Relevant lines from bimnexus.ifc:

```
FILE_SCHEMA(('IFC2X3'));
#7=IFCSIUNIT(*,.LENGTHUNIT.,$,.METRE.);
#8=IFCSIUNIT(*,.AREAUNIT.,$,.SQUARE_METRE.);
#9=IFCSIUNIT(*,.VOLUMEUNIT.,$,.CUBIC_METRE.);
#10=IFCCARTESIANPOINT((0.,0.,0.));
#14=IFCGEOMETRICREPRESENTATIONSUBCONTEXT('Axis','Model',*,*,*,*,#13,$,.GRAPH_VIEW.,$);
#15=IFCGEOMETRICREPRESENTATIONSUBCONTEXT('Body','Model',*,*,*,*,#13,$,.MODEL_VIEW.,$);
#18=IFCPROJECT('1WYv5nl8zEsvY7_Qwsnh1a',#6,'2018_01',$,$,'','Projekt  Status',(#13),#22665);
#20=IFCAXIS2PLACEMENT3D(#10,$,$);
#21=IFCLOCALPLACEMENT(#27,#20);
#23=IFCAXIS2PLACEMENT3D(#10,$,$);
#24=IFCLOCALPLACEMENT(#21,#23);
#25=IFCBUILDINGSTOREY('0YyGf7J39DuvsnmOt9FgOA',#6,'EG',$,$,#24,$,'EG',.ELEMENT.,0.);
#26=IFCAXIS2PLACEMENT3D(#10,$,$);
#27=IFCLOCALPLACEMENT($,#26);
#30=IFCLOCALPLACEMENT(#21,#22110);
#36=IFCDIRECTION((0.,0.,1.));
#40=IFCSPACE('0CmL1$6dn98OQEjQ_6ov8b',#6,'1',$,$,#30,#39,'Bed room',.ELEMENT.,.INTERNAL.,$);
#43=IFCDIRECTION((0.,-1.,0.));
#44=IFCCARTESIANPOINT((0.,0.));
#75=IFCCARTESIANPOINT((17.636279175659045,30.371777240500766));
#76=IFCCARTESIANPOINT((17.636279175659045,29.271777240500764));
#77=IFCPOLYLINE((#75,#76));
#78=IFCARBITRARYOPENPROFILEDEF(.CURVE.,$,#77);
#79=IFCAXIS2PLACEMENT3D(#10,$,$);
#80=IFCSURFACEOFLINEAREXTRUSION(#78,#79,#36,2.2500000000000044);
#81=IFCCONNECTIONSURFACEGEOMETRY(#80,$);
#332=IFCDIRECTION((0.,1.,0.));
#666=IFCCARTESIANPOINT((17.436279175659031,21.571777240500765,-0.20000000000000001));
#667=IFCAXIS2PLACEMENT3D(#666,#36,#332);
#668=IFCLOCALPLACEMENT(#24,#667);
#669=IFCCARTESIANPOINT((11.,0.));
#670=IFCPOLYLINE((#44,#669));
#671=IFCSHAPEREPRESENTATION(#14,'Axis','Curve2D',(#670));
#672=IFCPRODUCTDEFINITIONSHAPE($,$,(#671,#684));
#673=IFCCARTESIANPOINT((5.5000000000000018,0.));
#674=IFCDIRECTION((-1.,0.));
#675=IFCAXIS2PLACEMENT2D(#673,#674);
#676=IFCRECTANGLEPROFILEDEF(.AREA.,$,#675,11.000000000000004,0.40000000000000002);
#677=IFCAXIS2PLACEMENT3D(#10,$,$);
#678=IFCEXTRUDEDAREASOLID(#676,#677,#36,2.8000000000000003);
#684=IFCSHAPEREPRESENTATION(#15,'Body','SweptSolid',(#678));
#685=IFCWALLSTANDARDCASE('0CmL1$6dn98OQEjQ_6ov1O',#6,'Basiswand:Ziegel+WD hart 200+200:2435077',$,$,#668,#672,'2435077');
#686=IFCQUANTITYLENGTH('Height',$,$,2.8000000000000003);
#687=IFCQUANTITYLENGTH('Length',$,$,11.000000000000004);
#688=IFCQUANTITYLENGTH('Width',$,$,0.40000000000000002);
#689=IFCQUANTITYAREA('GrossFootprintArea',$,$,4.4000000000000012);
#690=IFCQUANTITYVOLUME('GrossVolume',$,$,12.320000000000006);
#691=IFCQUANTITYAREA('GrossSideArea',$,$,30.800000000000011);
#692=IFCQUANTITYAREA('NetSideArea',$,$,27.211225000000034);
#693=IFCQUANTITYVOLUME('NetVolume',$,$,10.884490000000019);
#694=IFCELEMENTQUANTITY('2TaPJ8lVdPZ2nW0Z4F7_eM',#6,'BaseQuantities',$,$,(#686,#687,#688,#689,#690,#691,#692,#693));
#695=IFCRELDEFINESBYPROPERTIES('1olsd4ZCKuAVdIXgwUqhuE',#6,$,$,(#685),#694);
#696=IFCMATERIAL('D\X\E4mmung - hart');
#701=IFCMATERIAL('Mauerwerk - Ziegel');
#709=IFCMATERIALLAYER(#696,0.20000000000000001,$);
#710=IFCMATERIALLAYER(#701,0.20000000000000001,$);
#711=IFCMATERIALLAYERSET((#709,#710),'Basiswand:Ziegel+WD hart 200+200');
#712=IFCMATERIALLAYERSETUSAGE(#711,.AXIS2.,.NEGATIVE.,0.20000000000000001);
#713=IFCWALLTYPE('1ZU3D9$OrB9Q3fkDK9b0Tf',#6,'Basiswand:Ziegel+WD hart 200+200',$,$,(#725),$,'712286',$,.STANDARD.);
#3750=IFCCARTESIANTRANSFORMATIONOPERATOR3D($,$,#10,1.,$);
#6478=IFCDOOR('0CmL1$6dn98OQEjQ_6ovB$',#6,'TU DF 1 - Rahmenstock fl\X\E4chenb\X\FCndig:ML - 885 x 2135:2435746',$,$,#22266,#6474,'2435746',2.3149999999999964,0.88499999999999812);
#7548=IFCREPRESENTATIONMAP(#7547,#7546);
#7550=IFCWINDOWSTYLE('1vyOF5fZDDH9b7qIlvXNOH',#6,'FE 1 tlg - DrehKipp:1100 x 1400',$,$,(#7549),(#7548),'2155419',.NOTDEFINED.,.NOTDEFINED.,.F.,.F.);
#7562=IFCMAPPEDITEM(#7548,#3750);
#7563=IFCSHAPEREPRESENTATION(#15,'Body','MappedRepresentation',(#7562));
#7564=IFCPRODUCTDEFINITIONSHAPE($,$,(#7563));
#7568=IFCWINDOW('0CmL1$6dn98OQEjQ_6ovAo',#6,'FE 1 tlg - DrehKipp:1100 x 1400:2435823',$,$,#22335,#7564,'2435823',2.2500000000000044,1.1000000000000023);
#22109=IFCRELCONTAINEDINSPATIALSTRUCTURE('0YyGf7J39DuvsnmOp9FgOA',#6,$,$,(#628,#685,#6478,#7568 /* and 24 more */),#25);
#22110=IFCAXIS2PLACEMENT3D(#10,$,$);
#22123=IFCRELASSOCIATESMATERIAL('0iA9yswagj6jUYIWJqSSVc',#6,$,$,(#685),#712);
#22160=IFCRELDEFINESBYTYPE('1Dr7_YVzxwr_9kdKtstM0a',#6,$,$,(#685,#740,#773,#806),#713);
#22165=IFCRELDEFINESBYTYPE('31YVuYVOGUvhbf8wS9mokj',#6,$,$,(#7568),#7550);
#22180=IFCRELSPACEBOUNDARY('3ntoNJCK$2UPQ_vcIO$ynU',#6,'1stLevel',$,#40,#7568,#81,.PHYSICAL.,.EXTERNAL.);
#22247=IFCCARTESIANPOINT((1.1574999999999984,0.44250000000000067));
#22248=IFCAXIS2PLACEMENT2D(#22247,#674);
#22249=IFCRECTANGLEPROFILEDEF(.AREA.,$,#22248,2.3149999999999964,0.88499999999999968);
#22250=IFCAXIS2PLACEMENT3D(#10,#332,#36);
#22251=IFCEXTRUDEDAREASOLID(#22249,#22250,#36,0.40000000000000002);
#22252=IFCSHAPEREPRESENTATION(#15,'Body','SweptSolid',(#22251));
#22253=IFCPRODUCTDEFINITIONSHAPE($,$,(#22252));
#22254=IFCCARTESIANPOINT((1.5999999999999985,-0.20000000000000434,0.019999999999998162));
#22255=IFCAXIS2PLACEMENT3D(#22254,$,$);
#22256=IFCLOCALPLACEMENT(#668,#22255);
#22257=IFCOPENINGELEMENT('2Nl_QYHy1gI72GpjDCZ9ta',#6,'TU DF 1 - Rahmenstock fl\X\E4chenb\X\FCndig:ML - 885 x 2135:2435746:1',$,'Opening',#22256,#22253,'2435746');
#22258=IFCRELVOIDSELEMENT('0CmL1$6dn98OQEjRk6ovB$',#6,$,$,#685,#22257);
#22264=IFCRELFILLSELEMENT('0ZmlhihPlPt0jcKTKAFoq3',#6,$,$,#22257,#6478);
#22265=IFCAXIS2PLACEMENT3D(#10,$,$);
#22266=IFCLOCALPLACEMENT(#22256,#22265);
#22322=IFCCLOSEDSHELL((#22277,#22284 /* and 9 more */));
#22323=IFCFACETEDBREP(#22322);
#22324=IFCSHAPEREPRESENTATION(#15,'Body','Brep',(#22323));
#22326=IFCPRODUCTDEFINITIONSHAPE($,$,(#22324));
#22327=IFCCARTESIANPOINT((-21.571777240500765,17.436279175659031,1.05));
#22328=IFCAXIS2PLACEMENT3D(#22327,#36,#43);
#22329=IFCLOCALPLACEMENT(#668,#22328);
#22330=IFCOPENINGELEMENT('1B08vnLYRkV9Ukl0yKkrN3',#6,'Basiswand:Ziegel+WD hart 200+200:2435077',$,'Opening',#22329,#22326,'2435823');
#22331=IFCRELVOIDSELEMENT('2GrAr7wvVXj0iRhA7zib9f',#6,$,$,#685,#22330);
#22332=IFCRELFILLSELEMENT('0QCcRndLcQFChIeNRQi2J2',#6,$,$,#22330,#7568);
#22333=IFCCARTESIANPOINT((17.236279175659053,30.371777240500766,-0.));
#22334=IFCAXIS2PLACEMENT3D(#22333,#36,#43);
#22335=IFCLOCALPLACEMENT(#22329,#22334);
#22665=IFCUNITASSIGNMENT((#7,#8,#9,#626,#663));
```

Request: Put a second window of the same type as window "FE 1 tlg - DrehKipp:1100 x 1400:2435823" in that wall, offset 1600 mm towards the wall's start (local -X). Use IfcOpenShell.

```python
import numpy as np
import ifcopenshell
import ifcopenshell.api.feature
import ifcopenshell.api.geometry
import ifcopenshell.api.pset
import ifcopenshell.api.root
import ifcopenshell.geom
import ifcopenshell.util.element
import ifcopenshell.util.placement
import ifcopenshell.util.shape
import ifcopenshell.util.unit

model = ifcopenshell.open("bimnexus.ifc")
unit_scale = ifcopenshell.util.unit.calculate_unit_scale(model)
area_scale = ifcopenshell.util.unit.calculate_unit_scale(model, "AREAUNIT")
volume_scale = ifcopenshell.util.unit.calculate_unit_scale(model, "VOLUMEUNIT")
settings = ifcopenshell.geom.settings()


def volume(element):
    """Net volume in cubic metres, openings subtracted."""
    shape = ifcopenshell.geom.create_shape(settings, element)
    return ifcopenshell.util.shape.get_volume(shape.geometry)


def reuse_history(source, copy):
    """copy_class also copies each property set's owner history, people and application; keep the originals."""
    for rel in copy.IsDefinedBy:
        if rel.is_a("IfcRelDefinesByProperties") and (history := rel.RelatingPropertyDefinition.OwnerHistory):
            rel.RelatingPropertyDefinition.OwnerHistory = source.OwnerHistory
            ifcopenshell.util.element.remove_deep2(model, history)


window = model.by_guid("0CmL1$6dn98OQEjQ_6ovAo")
opening = window.FillsVoids[0].RelatingOpeningElement
wall = opening.VoidsElements[0].RelatingBuildingElement
before = volume(wall)
shift = ifcopenshell.util.placement.get_local_placement(wall.ObjectPlacement)[:3, 0] * -1.6 / unit_scale

# copy_class copies the void relationship, type, container and properties, but no geometry.
new_opening = ifcopenshell.api.root.copy_class(model, product=opening)
new_opening.Representation = ifcopenshell.util.element.copy_deep(
    model, opening.Representation, exclude=["IfcGeometricRepresentationContext", "IfcRepresentationMap"]
)
new_opening.Name = "Basiswand:Ziegel+WD hart 200+200"
new_opening.Tag = None
new_window = ifcopenshell.api.root.copy_class(model, product=window)
new_window.Representation = ifcopenshell.util.element.copy_deep(
    model, window.Representation, exclude=["IfcGeometricRepresentationContext", "IfcRepresentationMap"]
)
new_window.Name = "FE 1 tlg - DrehKipp:1100 x 1400"
new_window.Tag = None
reuse_history(window, new_window)
fills = ifcopenshell.api.feature.add_filling(model, opening=new_opening, element=new_window)
fills.OwnerHistory = new_window.OwnerHistory  # required in IFC2X3

for old, new in ((opening, new_opening), (window, new_window)):
    matrix = ifcopenshell.util.placement.get_local_placement(old.ObjectPlacement)
    matrix[:3, 3] += shift
    ifcopenshell.api.geometry.edit_object_placement(model, product=new, matrix=matrix, is_si=False)

# The copied space boundaries still share their surfaces with the original.
for rel in new_window.ProvidesBoundaries:
    if rel.ConnectionGeometry:
        rel.ConnectionGeometry = ifcopenshell.util.element.copy_deep(model, rel.ConnectionGeometry)

# Space boundary surfaces are stored in each space's coordinates; move them too.
for rel in new_window.ProvidesBoundaries:
    if not rel.ConnectionGeometry:
        continue
    surface = rel.ConnectionGeometry.SurfaceOnRelatingElement
    space_matrix = ifcopenshell.util.placement.get_local_placement(rel.RelatingSpace.ObjectPlacement)
    point = np.array(surface.Position.Location.Coordinates) + space_matrix[:3, :3].T @ shift
    surface.Position = model.createIfcAxis2Placement3D(
        model.createIfcCartesianPoint(point.tolist()), surface.Position.Axis, surface.Position.RefDirection
    )

after = volume(wall)
thickness = 0.4  # wall thickness in metres

# Update the wall's stored quantities.
qto = model.by_id(ifcopenshell.util.element.get_pset(wall, "BaseQuantities", should_inherit=False)["id"])
ifcopenshell.api.pset.edit_qto(model, qto=qto, properties={
    "NetSideArea": after / thickness / area_scale,
    "NetVolume": after / volume_scale,
})

print(f"wall volume {before:.3f} -> {after:.3f} m3")

model.write("bimnexus-out.ifc")
```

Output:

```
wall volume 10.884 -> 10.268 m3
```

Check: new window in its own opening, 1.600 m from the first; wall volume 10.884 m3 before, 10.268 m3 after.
